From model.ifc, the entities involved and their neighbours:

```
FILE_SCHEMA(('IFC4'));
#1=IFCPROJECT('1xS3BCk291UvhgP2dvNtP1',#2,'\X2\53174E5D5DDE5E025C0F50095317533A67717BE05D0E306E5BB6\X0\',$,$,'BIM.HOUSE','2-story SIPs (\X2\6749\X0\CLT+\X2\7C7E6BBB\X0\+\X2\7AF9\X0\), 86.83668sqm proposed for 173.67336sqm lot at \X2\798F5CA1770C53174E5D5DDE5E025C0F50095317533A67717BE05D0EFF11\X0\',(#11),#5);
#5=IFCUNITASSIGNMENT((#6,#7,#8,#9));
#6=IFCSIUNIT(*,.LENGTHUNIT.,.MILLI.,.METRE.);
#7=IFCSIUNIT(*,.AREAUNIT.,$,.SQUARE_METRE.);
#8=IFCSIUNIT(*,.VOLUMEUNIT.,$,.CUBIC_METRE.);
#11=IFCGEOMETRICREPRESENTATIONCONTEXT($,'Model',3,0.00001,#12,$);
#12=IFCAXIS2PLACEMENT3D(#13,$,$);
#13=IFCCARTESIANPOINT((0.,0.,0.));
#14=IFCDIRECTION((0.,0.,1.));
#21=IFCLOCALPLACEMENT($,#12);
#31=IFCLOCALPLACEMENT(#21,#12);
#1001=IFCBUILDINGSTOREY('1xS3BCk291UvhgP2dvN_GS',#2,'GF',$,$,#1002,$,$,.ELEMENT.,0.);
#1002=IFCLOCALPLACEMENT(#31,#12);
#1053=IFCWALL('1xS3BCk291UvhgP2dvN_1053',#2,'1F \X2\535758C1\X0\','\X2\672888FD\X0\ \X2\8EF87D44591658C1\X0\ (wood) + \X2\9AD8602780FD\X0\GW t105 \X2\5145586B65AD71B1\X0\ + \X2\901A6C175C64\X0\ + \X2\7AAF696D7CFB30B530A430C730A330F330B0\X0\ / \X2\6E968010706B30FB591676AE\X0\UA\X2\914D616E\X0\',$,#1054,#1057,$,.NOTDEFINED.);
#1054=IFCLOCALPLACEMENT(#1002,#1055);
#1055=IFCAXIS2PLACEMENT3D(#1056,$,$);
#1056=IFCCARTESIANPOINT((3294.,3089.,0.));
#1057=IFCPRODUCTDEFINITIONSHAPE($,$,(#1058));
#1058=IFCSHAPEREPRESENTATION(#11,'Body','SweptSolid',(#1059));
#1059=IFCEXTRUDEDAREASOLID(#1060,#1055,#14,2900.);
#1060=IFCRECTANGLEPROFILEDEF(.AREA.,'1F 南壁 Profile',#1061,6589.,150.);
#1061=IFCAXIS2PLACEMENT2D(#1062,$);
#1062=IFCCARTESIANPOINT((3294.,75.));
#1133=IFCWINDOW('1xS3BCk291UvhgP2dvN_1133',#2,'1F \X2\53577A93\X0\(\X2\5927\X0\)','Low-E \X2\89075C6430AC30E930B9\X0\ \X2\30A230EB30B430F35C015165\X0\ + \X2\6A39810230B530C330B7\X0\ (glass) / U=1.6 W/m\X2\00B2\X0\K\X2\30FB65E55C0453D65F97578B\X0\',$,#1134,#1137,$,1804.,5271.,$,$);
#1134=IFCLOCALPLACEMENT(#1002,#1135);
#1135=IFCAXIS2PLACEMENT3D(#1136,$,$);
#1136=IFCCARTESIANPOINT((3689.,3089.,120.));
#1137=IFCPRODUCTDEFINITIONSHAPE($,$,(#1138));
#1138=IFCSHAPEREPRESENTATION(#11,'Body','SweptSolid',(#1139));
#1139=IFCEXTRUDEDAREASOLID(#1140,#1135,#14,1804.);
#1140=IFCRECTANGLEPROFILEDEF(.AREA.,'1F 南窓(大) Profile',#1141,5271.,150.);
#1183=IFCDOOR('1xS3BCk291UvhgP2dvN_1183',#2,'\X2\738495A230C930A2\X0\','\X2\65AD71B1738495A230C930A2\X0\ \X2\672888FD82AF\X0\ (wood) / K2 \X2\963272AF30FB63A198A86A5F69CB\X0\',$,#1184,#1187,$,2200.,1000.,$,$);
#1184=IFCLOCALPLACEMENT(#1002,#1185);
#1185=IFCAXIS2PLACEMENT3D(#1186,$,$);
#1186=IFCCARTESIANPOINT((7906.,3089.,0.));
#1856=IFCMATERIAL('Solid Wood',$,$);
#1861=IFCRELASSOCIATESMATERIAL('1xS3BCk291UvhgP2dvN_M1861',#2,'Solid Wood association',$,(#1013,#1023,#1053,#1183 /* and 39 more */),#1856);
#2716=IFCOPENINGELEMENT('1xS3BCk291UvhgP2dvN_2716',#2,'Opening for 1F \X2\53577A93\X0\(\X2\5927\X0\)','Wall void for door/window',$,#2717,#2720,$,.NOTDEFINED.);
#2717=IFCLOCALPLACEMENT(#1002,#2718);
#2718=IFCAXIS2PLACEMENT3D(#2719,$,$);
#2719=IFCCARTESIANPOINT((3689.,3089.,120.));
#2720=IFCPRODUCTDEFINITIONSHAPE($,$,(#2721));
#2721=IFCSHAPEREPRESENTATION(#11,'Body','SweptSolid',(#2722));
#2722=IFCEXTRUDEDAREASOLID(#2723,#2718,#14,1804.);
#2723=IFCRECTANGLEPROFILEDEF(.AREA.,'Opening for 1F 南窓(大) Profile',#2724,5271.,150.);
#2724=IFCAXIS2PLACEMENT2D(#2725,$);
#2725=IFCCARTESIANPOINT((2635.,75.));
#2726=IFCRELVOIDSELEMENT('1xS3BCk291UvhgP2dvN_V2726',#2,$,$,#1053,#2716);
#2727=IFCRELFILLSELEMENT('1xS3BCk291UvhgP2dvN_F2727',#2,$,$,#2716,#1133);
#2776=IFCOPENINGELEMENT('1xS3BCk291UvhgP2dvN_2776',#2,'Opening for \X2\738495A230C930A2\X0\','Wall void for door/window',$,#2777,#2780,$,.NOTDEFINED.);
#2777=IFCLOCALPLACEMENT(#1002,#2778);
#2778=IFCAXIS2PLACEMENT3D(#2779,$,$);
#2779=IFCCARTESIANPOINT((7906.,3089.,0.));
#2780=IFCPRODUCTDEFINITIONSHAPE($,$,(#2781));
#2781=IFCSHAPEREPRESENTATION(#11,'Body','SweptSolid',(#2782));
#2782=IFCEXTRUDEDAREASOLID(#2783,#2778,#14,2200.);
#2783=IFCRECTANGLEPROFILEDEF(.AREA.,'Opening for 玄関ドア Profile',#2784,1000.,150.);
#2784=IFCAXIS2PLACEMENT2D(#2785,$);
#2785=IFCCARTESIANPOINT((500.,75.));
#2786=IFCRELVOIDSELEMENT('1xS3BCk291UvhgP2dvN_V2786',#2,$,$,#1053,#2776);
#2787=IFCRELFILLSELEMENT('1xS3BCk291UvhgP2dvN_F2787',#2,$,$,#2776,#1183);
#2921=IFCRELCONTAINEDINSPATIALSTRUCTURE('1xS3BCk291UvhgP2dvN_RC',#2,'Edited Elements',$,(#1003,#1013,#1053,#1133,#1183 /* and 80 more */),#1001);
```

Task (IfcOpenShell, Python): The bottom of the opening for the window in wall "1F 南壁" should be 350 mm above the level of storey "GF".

```python
import numpy as np
import ifcopenshell
import ifcopenshell.api.geometry
import ifcopenshell.geom
import ifcopenshell.util.element
import ifcopenshell.util.placement
import ifcopenshell.util.shape
import ifcopenshell.util.unit

model = ifcopenshell.open("model.ifc")
unit_scale = ifcopenshell.util.unit.calculate_unit_scale(model)

window = model.by_guid("1xS3BCk291UvhgP2dvN_1133")
opening = window.FillsVoids[0].RelatingOpeningElement
storey = ifcopenshell.util.element.get_container(window, ifc_class="IfcBuildingStorey")
level = ifcopenshell.util.placement.get_local_placement(storey.ObjectPlacement)[2, 3]

# The opening's origin need not be at the sill, so measure its lowest point.
shape = ifcopenshell.geom.create_shape(ifcopenshell.geom.settings(), opening)
bottom = ifcopenshell.util.shape.get_shape_bottom_elevation(shape, shape.geometry) / unit_scale
dz = level + 350.0 - bottom

shift = np.array([0.0, 0.0, dz])
# The window is not placed relative to its opening, so move both.
for product in (opening, window):
    matrix = ifcopenshell.util.placement.get_local_placement(product.ObjectPlacement)
    matrix[:3, 3] += shift
    ifcopenshell.api.geometry.edit_object_placement(model, product=product, matrix=matrix, is_si=False)

print(f"moved by {dz * unit_scale:+.3f} m")

model.write("model_edited.ifc")
```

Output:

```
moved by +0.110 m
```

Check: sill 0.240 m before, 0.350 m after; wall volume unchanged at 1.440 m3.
